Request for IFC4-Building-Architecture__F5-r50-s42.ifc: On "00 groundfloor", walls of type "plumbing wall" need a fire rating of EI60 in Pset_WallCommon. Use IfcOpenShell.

First a look at what the model holds.

```python
import ifcopenshell
import ifcopenshell.util.element

model = ifcopenshell.open("IFC4-Building-Architecture__F5-r50-s42.ifc")
print(model.schema)
storey = next(s for s in model.by_type("IfcBuildingStorey") if s.Name == "00 groundfloor")
walls = [e for e in ifcopenshell.util.element.get_decomposition(storey) if e.is_a("IfcWall")]
seen = {}
for e in walls:
    element_type = ifcopenshell.util.element.get_type(e)
    key = (element_type.Name if element_type != e and element_type else None, ifcopenshell.util.element.get_pset(e, "Pset_WallCommon", "FireRating"))
    seen[key] = seen.get(key, 0) + 1
for (name, value), count in sorted(seen.items(), key=str):
    print(count, "x", name, "|", value)
```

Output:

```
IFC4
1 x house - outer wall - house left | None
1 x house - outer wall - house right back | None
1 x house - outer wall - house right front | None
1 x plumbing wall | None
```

```python
import ifcopenshell
import ifcopenshell.api.pset
import ifcopenshell.util.element

model = ifcopenshell.open("IFC4-Building-Architecture__F5-r50-s42.ifc")

storey = next(s for s in model.by_type("IfcBuildingStorey") if s.Name == "00 groundfloor")
walls = [e for e in ifcopenshell.util.element.get_decomposition(storey) if e.is_a("IfcWall")]

count = 0
for e in walls:
    element_type = ifcopenshell.util.element.get_type(e)
    if element_type in (None, e) or element_type.Name != "plumbing wall":
        continue
    # add_pset returns the element's existing set when there is one.
    pset = ifcopenshell.api.pset.add_pset(model, product=e, name="Pset_WallCommon")
    ifcopenshell.api.pset.edit_pset(model, pset=pset, properties={"FireRating": "EI60"})
    count += 1

print(count, "walls updated")

model.write("IFC4-Building-Architecture__F5-r50-s42_v2.ifc")
```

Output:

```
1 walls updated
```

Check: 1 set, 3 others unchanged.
